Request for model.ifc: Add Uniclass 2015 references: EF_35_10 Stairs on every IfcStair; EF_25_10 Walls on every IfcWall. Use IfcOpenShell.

First a look at what the model holds.

```python
import ifcopenshell

model = ifcopenshell.open("model.ifc")
print(model.schema)
print("classifications:", [c.Name for c in model.by_type("IfcClassification")])
for ifc_class in ("IfcDoor", "IfcRoof", "IfcStair", "IfcWall", "IfcWindow"):
    print(ifc_class, len(model.by_type(ifc_class)))
```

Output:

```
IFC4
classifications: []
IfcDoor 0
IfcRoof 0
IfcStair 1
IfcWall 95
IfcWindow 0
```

```python
import ifcopenshell
import ifcopenshell.api.classification

model = ifcopenshell.open("model.ifc")

system = ifcopenshell.api.classification.add_classification(model, classification="Uniclass 2015")

codes = {
    "IfcStair": ("EF_35_10", "Stairs"),
    "IfcWall": ("EF_25_10", "Walls"),
}
for ifc_class, (code, name) in codes.items():
    products = model.by_type(ifc_class)
    ifcopenshell.api.classification.add_reference(
        model, products=products, classification=system, identification=code, name=name
    )
    print(code, len(products))

model.write("model_updated.ifc")
```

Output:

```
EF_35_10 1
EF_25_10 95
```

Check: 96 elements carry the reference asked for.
